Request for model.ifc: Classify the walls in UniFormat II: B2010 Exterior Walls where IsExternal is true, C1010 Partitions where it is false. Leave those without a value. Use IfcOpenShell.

First a look at what the model holds.

```python
import ifcopenshell
import ifcopenshell.util.element

model = ifcopenshell.open("model.ifc")
print(model.schema)
print("classifications:", [c.Name for c in model.by_type("IfcClassification")])
values = [ifcopenshell.util.element.get_pset(e, "Pset_WallCommon", "IsExternal") for e in model.by_type("IfcWall")]
for value in (True, False, None):
    print("IsExternal", value, values.count(value))
```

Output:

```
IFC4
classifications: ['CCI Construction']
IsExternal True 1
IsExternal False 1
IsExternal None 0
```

```python
import ifcopenshell
import ifcopenshell.api.classification
import ifcopenshell.util.element

model = ifcopenshell.open("model.ifc")

system = ifcopenshell.api.classification.add_classification(model, classification="UniFormat II")

walls = model.by_type("IfcWall")
external = {e: ifcopenshell.util.element.get_pset(e, "Pset_WallCommon", "IsExternal") for e in walls}
for flag, code, name in ((True, "B2010", "Exterior Walls"), (False, "C1010", "Partitions")):
    products = [e for e in walls if external[e] is flag]
    ifcopenshell.api.classification.add_reference(
        model, products=products, classification=system, identification=code, name=name
    )
    print(code, len(products))

model.write("model_v2.ifc")
```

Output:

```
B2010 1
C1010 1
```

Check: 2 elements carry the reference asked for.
